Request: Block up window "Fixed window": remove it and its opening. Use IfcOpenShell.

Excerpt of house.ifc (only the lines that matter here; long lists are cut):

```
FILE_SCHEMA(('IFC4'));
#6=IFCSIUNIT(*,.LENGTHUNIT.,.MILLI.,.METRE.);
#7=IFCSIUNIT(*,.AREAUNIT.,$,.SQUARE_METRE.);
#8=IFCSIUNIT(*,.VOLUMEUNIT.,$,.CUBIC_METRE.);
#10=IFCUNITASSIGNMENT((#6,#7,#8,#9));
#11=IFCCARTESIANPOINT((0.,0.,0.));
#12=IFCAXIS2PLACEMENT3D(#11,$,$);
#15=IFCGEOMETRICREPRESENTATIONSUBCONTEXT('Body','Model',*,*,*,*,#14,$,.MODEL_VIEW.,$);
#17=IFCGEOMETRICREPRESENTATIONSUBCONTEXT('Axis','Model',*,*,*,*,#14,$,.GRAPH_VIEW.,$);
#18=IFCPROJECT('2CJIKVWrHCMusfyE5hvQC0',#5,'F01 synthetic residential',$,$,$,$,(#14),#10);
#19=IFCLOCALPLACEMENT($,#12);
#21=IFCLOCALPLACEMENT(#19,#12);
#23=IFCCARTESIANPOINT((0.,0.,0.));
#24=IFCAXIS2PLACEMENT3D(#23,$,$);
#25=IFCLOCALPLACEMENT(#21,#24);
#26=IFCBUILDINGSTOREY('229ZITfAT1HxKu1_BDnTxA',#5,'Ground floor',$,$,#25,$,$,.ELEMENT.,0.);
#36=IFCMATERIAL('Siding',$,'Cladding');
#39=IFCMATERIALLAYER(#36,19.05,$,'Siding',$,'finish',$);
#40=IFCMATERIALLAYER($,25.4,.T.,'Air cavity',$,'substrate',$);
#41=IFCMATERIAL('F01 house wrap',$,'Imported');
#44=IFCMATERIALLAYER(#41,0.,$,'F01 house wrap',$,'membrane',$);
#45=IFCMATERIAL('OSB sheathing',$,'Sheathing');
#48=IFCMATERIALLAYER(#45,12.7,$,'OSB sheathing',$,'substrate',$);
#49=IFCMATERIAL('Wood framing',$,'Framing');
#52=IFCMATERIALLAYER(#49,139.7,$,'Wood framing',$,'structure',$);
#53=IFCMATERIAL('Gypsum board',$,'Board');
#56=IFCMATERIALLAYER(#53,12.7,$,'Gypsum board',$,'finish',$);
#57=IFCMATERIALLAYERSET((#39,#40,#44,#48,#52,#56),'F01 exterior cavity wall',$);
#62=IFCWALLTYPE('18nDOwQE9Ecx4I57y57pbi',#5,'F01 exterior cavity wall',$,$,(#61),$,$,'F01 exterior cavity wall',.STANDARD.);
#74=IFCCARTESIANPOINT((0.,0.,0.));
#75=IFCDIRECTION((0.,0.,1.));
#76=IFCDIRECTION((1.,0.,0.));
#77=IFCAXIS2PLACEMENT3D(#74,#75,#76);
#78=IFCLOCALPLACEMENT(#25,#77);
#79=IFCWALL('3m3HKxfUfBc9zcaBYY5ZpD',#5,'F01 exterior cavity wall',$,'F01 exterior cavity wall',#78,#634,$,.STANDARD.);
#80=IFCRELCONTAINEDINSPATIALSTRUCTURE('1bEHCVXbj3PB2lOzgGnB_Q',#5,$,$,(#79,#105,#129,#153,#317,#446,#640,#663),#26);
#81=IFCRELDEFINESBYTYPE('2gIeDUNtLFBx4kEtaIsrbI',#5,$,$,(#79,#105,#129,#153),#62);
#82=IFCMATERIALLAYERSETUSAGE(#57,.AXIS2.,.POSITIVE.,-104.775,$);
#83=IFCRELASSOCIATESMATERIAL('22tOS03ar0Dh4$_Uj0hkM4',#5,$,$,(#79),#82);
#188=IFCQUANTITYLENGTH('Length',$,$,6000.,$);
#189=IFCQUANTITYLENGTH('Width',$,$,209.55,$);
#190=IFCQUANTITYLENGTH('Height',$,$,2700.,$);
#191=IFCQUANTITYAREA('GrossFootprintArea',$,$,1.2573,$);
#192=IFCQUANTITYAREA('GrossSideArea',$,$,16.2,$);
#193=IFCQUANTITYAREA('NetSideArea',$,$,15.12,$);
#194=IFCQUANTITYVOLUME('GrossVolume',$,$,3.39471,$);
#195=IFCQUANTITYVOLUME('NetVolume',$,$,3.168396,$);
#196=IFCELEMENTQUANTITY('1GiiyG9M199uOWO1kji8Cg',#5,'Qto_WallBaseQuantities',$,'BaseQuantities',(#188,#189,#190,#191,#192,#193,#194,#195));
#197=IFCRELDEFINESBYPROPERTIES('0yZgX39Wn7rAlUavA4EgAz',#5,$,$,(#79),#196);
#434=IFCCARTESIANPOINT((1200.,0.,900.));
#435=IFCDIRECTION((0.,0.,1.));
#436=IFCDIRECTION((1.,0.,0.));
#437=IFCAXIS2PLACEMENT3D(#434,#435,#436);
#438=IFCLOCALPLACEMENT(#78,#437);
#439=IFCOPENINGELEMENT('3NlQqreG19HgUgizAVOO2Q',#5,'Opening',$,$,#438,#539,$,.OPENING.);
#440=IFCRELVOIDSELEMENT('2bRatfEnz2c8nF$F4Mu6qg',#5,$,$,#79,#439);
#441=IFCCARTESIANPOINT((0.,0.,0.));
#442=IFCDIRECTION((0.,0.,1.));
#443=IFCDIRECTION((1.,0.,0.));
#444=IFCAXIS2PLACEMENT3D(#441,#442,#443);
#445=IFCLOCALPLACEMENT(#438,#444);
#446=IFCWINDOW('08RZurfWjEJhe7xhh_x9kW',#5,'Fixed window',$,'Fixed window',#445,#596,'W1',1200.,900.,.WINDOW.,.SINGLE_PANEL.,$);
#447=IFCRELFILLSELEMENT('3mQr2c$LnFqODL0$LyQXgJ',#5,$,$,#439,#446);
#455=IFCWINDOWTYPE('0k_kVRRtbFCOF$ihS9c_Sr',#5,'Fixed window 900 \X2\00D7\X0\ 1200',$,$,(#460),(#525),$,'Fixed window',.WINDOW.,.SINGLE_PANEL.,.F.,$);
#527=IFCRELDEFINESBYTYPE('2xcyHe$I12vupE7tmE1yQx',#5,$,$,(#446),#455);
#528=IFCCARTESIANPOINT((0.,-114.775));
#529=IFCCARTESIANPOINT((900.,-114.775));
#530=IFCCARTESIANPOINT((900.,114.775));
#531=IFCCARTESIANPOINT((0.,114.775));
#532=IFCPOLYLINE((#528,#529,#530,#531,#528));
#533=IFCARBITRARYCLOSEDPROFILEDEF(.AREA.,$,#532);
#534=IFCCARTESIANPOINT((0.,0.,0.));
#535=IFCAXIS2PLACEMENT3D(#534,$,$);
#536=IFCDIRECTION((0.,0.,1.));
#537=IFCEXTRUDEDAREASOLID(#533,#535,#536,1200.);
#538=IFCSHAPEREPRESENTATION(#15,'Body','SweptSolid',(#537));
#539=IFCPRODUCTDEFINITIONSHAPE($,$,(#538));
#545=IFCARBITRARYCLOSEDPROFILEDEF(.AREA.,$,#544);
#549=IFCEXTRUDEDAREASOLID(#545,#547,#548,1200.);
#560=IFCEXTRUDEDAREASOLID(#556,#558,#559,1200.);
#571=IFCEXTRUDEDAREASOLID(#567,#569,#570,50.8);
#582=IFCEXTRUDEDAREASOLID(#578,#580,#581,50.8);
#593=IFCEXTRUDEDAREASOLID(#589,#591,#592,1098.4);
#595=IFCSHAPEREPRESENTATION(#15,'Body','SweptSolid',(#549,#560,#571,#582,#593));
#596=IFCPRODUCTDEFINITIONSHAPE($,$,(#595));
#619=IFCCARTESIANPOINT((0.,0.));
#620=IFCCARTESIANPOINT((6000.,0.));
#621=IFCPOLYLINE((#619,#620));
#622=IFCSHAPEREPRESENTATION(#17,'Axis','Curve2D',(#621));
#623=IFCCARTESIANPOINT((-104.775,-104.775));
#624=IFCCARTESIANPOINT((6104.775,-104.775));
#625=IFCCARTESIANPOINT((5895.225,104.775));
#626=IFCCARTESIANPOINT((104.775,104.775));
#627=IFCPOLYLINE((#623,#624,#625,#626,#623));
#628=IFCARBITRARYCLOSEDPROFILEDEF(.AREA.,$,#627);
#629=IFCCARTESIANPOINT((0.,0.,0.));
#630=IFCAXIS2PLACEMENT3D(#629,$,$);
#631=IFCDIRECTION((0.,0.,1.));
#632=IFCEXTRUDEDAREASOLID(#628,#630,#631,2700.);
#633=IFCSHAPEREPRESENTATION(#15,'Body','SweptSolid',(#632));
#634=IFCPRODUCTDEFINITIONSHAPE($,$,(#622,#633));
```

```python
import ifcopenshell
import ifcopenshell.api.feature
import ifcopenshell.api.pset
import ifcopenshell.api.root
import ifcopenshell.geom
import ifcopenshell.util.element
import ifcopenshell.util.shape
import ifcopenshell.util.unit

model = ifcopenshell.open("house.ifc")
area_scale = ifcopenshell.util.unit.calculate_unit_scale(model, "AREAUNIT")
volume_scale = ifcopenshell.util.unit.calculate_unit_scale(model, "VOLUMEUNIT")
settings = ifcopenshell.geom.settings()


def volume(element):
    """Net volume in cubic metres, openings subtracted."""
    shape = ifcopenshell.geom.create_shape(settings, element)
    return ifcopenshell.util.shape.get_volume(shape.geometry)


window = model.by_guid("08RZurfWjEJhe7xhh_x9kW")
opening = window.FillsVoids[0].RelatingOpeningElement
wall = opening.VoidsElements[0].RelatingBuildingElement
before = volume(wall)

ifcopenshell.api.root.remove_product(model, product=window)
ifcopenshell.api.feature.remove_feature(model, feature=opening)

after = volume(wall)
thickness = 0.2096  # wall thickness in metres

# Update the wall's stored quantities.
qto = model.by_id(ifcopenshell.util.element.get_pset(wall, "Qto_WallBaseQuantities", should_inherit=False)["id"])
ifcopenshell.api.pset.edit_qto(model, qto=qto, properties={
    "NetSideArea": after / thickness / area_scale,
    "NetVolume": after / volume_scale,
})

print(f"wall volume {before:.3f} -> {after:.3f} m3")

model.write("house-out.ifc")
```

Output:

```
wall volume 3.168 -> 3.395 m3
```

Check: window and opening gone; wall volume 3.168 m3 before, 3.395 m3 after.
